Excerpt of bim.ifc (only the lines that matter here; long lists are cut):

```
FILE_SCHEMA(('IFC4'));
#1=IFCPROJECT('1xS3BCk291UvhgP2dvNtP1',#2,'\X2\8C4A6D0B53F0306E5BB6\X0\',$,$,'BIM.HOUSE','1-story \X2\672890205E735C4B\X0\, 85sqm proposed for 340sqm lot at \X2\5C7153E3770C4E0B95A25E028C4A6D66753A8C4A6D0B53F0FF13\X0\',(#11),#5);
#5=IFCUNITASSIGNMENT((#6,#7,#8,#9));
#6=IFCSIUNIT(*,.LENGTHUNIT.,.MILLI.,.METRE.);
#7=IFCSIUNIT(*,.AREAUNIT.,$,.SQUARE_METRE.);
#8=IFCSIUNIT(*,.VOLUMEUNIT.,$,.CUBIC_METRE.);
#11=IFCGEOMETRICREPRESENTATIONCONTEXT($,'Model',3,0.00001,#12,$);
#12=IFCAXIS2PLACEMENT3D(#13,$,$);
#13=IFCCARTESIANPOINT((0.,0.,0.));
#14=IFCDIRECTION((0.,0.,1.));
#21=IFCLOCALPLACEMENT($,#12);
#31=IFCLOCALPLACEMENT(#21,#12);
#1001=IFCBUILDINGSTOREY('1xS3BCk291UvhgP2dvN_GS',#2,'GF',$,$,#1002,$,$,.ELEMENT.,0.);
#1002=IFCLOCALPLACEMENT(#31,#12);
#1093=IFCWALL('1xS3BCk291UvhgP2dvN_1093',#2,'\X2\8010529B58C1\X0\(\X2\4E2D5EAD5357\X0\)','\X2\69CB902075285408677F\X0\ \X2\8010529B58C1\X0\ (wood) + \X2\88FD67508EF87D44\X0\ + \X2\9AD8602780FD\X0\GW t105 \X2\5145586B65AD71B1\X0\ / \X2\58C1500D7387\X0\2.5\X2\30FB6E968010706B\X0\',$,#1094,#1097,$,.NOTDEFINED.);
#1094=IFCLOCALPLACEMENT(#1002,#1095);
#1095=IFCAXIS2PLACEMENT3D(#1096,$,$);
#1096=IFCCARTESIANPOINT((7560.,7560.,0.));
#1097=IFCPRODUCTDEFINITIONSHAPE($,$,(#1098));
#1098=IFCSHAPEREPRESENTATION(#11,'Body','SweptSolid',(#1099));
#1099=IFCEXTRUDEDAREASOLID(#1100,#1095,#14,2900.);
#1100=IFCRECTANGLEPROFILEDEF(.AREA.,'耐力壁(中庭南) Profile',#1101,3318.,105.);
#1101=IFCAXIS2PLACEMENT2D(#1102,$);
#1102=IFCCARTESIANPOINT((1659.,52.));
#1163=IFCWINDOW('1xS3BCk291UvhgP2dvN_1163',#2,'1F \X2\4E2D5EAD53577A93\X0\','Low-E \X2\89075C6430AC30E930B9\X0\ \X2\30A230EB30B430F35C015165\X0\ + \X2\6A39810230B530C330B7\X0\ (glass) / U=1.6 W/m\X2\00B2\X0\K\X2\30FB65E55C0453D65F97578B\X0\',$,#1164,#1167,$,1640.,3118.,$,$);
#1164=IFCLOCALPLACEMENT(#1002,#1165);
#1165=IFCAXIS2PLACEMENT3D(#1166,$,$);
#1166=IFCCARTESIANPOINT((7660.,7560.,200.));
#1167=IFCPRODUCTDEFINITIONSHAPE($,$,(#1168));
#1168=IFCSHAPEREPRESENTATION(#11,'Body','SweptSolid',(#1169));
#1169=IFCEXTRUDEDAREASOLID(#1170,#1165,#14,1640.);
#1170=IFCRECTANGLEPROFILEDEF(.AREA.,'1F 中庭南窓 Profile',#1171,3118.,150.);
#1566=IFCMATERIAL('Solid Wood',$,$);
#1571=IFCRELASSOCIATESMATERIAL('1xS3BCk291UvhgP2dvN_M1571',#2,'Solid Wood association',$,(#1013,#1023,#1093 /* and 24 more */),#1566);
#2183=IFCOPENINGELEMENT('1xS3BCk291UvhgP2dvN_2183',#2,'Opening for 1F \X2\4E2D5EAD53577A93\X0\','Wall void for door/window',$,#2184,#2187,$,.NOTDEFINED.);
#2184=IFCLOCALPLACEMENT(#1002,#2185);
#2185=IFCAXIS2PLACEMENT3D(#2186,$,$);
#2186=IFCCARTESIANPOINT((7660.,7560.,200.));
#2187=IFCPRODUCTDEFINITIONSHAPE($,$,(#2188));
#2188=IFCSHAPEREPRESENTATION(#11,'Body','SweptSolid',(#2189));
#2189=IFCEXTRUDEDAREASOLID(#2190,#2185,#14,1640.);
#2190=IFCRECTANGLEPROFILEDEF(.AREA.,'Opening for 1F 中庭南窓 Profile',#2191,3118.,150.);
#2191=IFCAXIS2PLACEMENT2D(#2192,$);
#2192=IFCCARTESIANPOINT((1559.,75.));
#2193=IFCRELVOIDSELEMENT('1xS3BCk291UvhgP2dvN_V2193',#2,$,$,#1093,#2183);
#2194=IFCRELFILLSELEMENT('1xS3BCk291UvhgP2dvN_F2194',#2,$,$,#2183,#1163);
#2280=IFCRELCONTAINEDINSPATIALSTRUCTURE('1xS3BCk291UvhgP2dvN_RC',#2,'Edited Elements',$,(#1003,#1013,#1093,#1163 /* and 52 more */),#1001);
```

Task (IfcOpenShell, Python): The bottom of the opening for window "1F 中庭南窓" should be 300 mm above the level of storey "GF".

```python
import numpy as np
import ifcopenshell
import ifcopenshell.api.geometry
import ifcopenshell.geom
import ifcopenshell.util.element
import ifcopenshell.util.placement
import ifcopenshell.util.shape
import ifcopenshell.util.unit

model = ifcopenshell.open("bim.ifc")
unit_scale = ifcopenshell.util.unit.calculate_unit_scale(model)

window = model.by_id(1163)
opening = window.FillsVoids[0].RelatingOpeningElement
storey = ifcopenshell.util.element.get_container(window, ifc_class="IfcBuildingStorey")
level = ifcopenshell.util.placement.get_local_placement(storey.ObjectPlacement)[2, 3]

# The opening's origin need not be at the sill, so measure its lowest point.
shape = ifcopenshell.geom.create_shape(ifcopenshell.geom.settings(), opening)
bottom = ifcopenshell.util.shape.get_shape_bottom_elevation(shape, shape.geometry) / unit_scale
dz = level + 0.3 / unit_scale - bottom

shift = np.array([0.0, 0.0, dz])
# The window is not placed relative to its opening, so move both.
for product in (opening, window):
    matrix = ifcopenshell.util.placement.get_local_placement(product.ObjectPlacement)
    matrix[:3, 3] += shift
    ifcopenshell.api.geometry.edit_object_placement(model, product=product, matrix=matrix, is_si=False)

print(f"moved by {dz * unit_scale:+.3f} m")

model.write("bim_rev.ifc")
```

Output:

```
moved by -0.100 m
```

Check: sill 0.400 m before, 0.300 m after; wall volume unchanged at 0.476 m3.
